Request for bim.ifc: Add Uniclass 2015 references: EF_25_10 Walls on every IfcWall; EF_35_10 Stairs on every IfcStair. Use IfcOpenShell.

First a look at what the model holds.

```python
import ifcopenshell

model = ifcopenshell.open("bim.ifc")
print(model.schema)
print("classifications:", [c.Name for c in model.by_type("IfcClassification")])
for ifc_class in ("IfcDoor", "IfcRoof", "IfcStair", "IfcWall", "IfcWindow"):
    print(ifc_class, len(model.by_type(ifc_class)))
```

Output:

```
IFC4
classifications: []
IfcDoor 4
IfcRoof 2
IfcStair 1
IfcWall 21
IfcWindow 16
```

```python
import ifcopenshell
import ifcopenshell.api.classification

model = ifcopenshell.open("bim.ifc")

system = ifcopenshell.api.classification.add_classification(model, classification="Uniclass 2015")

codes = {
    "IfcWall": ("EF_25_10", "Walls"),
    "IfcStair": ("EF_35_10", "Stairs"),
}
for ifc_class, (code, name) in codes.items():
    products = model.by_type(ifc_class)
    ifcopenshell.api.classification.add_reference(
        model, products=products, classification=system, identification=code, name=name
    )
    print(code, len(products))

model.write("bim_updated.ifc")
```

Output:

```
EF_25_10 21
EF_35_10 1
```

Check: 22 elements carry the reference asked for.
